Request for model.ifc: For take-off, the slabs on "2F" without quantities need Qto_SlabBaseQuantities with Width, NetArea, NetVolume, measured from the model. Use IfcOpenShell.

First a look at what the model holds.

```python
import ifcopenshell
import ifcopenshell.util.element
import ifcopenshell.util.unit

model = ifcopenshell.open("model.ifc")
print(model.schema)
for unit_type in ("LENGTHUNIT", "AREAUNIT", "VOLUMEUNIT"):
    print(unit_type, ifcopenshell.util.unit.calculate_unit_scale(model, unit_type))
storey = next(s for s in model.by_type("IfcBuildingStorey") if s.Name == "2F")
slabs = [e for e in ifcopenshell.util.element.get_decomposition(storey) if e.is_a("IfcSlab")]
for e in sorted(slabs, key=lambda e: e.id()):
    print(e.id(), e.is_a(), e.Name, list(ifcopenshell.util.element.get_psets(e, qtos_only=True)), sep=" | ")
```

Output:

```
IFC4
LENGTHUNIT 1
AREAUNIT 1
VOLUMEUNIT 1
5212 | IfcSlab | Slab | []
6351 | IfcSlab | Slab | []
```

```python
import ifcopenshell
import ifcopenshell.api.pset
import ifcopenshell.geom
import ifcopenshell.util.element
import ifcopenshell.util.shape
import ifcopenshell.util.unit

model = ifcopenshell.open("model.ifc")
unit_scale = ifcopenshell.util.unit.calculate_unit_scale(model)
area_scale = ifcopenshell.util.unit.calculate_unit_scale(model, "AREAUNIT")
volume_scale = ifcopenshell.util.unit.calculate_unit_scale(model, "VOLUMEUNIT")
settings = ifcopenshell.geom.settings()

storey = next(s for s in model.by_type("IfcBuildingStorey") if s.Name == "2F")
slabs = [e for e in ifcopenshell.util.element.get_decomposition(storey) if e.is_a("IfcSlab")]

for e in sorted(slabs, key=lambda e: e.id()):
    if ifcopenshell.util.element.get_psets(e, qtos_only=True, should_inherit=False):
        continue
    # Geometry comes back in metres, in the element's own axes.
    shape = ifcopenshell.geom.create_shape(settings, e)
    values = {
        "Width": ifcopenshell.util.shape.get_z(shape.geometry) / unit_scale,
        "NetArea": ifcopenshell.util.shape.get_footprint_area(shape.geometry) / area_scale,
        "NetVolume": ifcopenshell.util.shape.get_volume(shape.geometry) / volume_scale,
    }
    qto = ifcopenshell.api.pset.add_qto(model, product=e, name="Qto_SlabBaseQuantities")
    ifcopenshell.api.pset.edit_qto(model, qto=qto, properties=values)
    print(e.id(), {k: round(v, 3) for k, v in values.items()})

model.write("model-out.ifc")
```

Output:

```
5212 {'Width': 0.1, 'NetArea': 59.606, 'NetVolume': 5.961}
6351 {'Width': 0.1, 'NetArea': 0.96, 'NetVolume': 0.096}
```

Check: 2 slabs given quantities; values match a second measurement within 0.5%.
